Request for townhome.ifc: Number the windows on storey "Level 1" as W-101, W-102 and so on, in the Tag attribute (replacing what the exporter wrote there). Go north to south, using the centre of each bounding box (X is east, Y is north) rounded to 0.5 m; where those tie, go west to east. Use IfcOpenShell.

First a look at what the model holds.

```python
import ifcopenshell
import ifcopenshell.util.element
import ifcopenshell.util.placement

model = ifcopenshell.open("townhome.ifc")
print(model.schema)
storey = next(s for s in model.by_type("IfcBuildingStorey") if s.Name == "Level 1")
windows = [e for e in ifcopenshell.util.element.get_decomposition(storey) if e.is_a("IfcWindow")]
for e in sorted(windows, key=lambda e: e.id()):
    origin = ifcopenshell.util.placement.get_local_placement(e.ObjectPlacement)[:3, 3]
    print(e.id(), e.Tag, e.Name, origin.round(2) + 0.0, sep=" | ")
```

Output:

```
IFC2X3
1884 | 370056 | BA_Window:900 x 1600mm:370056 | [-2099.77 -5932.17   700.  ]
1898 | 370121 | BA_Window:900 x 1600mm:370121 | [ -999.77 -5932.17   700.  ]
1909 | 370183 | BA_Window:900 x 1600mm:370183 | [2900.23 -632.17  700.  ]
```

```python
import ifcopenshell
import ifcopenshell.geom
import ifcopenshell.util.element
import ifcopenshell.util.shape

model = ifcopenshell.open("townhome.ifc")
settings = ifcopenshell.geom.settings()
settings.set("use-world-coords", True)


def centre(element):
    shape = ifcopenshell.geom.create_shape(settings, element)
    return ifcopenshell.util.shape.get_bbox_centroid(shape.geometry)


storey = next(s for s in model.by_type("IfcBuildingStorey") if s.Name == "Level 1")
windows = [e for e in ifcopenshell.util.element.get_decomposition(storey) if e.is_a("IfcWindow")]

# Insertion points can sit at a corner or the storey origin, so sort by the geometry (in metres).
centres = {e: centre(e) for e in windows}
windows.sort(key=lambda e: (-round(centres[e][1] / 0.5), centres[e][0]))

for i, e in enumerate(windows, start=1):
    number = f"W-1{i:02d}"
    e.Tag = number
    print(e.id(), number)

model.write("townhome_v2.ifc")
```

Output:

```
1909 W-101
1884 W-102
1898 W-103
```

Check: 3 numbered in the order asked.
